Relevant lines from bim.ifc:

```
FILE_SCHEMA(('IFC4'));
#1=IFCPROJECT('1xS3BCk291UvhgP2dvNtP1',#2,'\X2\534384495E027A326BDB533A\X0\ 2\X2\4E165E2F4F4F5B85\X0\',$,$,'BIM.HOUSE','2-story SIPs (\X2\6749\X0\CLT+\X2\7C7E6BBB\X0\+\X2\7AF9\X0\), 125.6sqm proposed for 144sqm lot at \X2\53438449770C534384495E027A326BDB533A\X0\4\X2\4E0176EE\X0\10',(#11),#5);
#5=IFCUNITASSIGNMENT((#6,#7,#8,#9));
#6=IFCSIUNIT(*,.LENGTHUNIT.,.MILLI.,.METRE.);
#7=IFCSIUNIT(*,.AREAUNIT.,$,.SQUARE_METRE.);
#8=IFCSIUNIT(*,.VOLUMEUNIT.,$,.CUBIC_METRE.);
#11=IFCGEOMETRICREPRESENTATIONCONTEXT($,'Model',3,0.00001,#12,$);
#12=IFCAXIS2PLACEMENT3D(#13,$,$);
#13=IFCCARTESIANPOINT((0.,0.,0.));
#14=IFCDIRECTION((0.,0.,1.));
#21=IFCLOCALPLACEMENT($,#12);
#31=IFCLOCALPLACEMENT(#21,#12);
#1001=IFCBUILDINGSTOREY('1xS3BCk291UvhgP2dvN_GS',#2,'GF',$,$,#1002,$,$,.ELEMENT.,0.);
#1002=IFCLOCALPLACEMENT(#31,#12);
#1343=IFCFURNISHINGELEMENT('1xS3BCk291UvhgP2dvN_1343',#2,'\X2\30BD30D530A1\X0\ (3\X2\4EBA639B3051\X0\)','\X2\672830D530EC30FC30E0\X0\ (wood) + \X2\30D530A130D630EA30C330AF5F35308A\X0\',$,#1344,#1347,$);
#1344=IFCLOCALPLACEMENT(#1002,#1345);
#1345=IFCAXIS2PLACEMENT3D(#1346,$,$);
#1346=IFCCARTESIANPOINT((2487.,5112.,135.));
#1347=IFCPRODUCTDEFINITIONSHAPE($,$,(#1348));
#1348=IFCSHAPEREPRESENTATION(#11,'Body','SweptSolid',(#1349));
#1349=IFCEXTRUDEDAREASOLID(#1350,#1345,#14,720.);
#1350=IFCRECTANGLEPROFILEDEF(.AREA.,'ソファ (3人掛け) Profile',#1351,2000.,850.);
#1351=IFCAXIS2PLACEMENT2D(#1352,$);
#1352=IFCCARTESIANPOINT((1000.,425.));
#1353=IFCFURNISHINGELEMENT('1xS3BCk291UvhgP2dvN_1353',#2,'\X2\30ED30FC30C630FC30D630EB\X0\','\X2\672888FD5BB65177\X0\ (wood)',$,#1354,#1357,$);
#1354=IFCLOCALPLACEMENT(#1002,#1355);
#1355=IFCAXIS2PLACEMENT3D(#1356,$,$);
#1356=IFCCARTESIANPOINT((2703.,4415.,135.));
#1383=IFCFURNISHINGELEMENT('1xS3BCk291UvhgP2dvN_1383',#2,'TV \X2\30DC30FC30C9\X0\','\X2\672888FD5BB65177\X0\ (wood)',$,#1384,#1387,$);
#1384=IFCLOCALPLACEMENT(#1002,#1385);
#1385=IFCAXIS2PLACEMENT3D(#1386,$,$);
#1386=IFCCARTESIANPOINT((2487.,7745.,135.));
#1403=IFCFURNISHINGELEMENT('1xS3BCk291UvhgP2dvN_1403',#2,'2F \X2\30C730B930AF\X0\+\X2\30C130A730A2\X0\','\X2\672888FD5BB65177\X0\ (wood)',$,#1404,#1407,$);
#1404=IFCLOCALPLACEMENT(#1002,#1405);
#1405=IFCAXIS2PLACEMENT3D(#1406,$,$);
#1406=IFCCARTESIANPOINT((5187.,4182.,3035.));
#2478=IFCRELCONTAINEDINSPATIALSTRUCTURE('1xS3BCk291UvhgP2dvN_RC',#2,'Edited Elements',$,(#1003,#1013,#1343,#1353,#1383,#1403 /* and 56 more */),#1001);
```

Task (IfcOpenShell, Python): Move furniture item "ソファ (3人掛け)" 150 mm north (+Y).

```python
import ifcopenshell
import ifcopenshell.api.geometry
import ifcopenshell.util.placement

model = ifcopenshell.open("bim.ifc")

item = model.by_id(1343)
matrix = ifcopenshell.util.placement.get_local_placement(item.ObjectPlacement)
matrix[1, 3] += 150.0
ifcopenshell.api.geometry.edit_object_placement(model, product=item, matrix=matrix, is_si=False)

print(ifcopenshell.util.placement.get_local_placement(item.ObjectPlacement).round(3) + 0.0)

model.write("bim_v2.ifc")
```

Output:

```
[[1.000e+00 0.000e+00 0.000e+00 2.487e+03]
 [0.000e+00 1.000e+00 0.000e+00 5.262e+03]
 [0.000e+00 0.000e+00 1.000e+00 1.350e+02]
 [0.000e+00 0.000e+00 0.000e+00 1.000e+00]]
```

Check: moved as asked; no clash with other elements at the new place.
